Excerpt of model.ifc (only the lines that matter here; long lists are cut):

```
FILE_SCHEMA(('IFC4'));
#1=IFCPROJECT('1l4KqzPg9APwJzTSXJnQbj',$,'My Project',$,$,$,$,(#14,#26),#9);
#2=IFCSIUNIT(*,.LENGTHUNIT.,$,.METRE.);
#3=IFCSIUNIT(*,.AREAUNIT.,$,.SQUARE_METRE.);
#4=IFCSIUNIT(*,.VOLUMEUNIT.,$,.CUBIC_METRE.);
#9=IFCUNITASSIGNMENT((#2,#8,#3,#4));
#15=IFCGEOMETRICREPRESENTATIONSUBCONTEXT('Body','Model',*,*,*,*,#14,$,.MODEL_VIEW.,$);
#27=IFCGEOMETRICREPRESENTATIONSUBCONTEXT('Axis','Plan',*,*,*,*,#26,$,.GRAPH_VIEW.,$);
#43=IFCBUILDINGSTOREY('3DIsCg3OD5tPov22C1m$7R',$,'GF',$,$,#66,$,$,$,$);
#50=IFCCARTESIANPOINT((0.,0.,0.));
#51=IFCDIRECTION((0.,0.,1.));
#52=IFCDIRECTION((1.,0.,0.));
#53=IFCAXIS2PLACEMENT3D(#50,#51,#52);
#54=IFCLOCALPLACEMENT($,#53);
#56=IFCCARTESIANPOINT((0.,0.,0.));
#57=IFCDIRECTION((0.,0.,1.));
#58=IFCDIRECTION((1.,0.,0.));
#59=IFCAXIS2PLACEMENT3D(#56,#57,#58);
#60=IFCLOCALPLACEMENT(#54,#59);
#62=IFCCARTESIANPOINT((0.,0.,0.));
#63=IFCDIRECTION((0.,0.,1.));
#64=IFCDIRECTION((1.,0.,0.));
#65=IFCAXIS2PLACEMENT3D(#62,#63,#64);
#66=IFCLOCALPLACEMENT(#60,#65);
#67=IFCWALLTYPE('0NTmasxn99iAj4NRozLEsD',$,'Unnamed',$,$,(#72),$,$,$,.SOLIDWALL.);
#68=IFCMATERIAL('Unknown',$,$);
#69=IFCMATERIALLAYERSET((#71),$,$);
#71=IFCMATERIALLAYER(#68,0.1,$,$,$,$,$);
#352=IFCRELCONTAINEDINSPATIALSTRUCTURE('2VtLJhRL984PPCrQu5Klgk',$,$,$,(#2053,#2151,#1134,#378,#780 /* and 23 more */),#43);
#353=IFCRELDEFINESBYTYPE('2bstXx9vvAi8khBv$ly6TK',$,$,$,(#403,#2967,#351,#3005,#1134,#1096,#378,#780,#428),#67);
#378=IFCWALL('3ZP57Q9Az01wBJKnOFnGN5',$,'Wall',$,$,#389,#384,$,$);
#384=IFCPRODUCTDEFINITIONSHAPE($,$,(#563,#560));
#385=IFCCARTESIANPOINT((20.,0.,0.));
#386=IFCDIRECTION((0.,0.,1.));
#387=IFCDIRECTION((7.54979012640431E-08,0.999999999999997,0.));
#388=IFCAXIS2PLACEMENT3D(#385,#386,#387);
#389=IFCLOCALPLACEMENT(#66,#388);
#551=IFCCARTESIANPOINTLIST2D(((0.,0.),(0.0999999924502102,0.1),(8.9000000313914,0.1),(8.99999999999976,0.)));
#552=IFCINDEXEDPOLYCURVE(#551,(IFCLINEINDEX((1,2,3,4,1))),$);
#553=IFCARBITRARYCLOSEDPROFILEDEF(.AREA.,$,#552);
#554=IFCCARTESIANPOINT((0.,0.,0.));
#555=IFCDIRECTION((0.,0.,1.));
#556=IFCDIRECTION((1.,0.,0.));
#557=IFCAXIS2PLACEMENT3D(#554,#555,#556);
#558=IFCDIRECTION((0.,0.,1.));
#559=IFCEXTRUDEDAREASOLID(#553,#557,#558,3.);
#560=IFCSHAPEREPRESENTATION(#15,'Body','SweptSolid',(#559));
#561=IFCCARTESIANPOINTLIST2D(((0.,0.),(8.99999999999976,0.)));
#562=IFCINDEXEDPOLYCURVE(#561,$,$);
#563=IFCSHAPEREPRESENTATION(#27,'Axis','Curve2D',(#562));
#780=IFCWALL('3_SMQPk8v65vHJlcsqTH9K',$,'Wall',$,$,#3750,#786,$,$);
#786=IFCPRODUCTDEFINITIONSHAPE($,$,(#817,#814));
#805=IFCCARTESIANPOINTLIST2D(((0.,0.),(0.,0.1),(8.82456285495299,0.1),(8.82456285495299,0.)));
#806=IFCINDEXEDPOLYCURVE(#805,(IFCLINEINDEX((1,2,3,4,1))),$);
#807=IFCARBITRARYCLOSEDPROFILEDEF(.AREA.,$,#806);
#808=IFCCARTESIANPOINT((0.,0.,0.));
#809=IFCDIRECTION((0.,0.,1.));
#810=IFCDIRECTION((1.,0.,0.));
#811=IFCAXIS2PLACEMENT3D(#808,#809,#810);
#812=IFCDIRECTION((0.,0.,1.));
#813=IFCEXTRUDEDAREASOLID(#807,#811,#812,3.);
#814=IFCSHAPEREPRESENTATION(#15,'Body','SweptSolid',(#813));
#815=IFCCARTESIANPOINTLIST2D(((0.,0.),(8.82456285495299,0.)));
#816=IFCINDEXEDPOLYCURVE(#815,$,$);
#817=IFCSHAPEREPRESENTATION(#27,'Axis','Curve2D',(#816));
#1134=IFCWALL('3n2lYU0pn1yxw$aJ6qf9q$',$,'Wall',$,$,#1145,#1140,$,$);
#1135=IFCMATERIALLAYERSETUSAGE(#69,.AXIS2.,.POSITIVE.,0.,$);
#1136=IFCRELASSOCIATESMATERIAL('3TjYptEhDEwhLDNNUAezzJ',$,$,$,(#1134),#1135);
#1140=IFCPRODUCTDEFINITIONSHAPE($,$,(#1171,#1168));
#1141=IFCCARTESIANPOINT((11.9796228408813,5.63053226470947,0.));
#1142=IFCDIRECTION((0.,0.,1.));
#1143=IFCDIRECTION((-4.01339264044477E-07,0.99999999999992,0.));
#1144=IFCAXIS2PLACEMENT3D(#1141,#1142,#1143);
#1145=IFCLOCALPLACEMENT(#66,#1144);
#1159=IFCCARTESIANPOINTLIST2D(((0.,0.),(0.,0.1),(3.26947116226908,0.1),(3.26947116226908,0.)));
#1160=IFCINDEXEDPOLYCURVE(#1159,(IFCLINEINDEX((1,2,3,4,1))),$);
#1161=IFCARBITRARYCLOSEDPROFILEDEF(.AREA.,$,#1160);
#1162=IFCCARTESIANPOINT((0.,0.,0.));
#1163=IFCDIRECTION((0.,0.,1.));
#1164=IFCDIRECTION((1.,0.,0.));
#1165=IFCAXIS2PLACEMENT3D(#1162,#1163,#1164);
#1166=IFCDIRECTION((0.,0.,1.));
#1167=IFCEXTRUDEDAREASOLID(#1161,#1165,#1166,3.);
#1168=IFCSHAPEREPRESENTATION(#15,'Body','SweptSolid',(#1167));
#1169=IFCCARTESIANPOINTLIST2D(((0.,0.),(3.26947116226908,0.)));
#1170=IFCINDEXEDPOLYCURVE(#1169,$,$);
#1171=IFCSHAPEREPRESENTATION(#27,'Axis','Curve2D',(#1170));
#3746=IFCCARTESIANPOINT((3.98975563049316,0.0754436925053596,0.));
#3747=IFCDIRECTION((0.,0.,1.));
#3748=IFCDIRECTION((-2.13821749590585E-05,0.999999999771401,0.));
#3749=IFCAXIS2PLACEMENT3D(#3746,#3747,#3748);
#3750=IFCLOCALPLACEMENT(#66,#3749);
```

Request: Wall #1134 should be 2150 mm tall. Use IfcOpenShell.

```python
import ifcopenshell
import ifcopenshell.geom
import ifcopenshell.util.representation
import ifcopenshell.util.shape

model = ifcopenshell.open("model.ifc")
settings = ifcopenshell.geom.settings()


def volume(element):
    """Net volume in cubic metres, openings subtracted."""
    shape = ifcopenshell.geom.create_shape(settings, element)
    return ifcopenshell.util.shape.get_volume(shape.geometry)


wall = model.by_guid("3n2lYU0pn1yxw$aJ6qf9q$")
before = volume(wall)

body = ifcopenshell.util.representation.get_representation(wall, "Model", "Body")
solid = body.Items[0]
old_height = solid.Depth
solid.Depth = 2.15
after = volume(wall)

print(f"height {old_height:g} -> {solid.Depth:g}, volume {before:.3f} -> {after:.3f} m3")

model.write("model_edited.ifc")
```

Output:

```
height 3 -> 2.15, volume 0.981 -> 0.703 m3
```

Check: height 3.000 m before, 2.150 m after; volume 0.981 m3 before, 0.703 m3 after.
